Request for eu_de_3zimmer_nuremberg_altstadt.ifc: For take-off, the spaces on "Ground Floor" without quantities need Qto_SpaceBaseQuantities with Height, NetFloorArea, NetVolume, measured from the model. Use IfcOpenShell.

First a look at what the model holds.

```python
import ifcopenshell
import ifcopenshell.util.element
import ifcopenshell.util.unit

model = ifcopenshell.open("eu_de_3zimmer_nuremberg_altstadt.ifc")
print(model.schema)
for unit_type in ("LENGTHUNIT", "AREAUNIT", "VOLUMEUNIT"):
    print(unit_type, ifcopenshell.util.unit.calculate_unit_scale(model, unit_type))
storey = next(s for s in model.by_type("IfcBuildingStorey") if s.Name == "Ground Floor")
spaces = [e for e in ifcopenshell.util.element.get_decomposition(storey) if e.is_a("IfcSpace")]
for e in sorted(spaces, key=lambda e: e.id()):
    print(e.id(), e.is_a(), e.Name, list(ifcopenshell.util.element.get_psets(e, qtos_only=True)), sep=" | ")
```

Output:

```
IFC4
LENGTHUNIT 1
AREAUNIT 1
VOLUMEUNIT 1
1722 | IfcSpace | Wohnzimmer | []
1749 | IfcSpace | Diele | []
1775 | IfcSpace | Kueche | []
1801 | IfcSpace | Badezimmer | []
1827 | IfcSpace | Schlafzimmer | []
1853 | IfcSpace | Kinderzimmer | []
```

```python
import ifcopenshell
import ifcopenshell.api.pset
import ifcopenshell.geom
import ifcopenshell.util.element
import ifcopenshell.util.shape
import ifcopenshell.util.unit

model = ifcopenshell.open("eu_de_3zimmer_nuremberg_altstadt.ifc")
unit_scale = ifcopenshell.util.unit.calculate_unit_scale(model)
area_scale = ifcopenshell.util.unit.calculate_unit_scale(model, "AREAUNIT")
volume_scale = ifcopenshell.util.unit.calculate_unit_scale(model, "VOLUMEUNIT")
settings = ifcopenshell.geom.settings()

storey = next(s for s in model.by_type("IfcBuildingStorey") if s.Name == "Ground Floor")
spaces = [e for e in ifcopenshell.util.element.get_decomposition(storey) if e.is_a("IfcSpace")]

for e in sorted(spaces, key=lambda e: e.id()):
    if ifcopenshell.util.element.get_psets(e, qtos_only=True, should_inherit=False):
        continue
    # Geometry comes back in metres, in the element's own axes.
    shape = ifcopenshell.geom.create_shape(settings, e)
    values = {
        "Height": ifcopenshell.util.shape.get_z(shape.geometry) / unit_scale,
        "NetFloorArea": ifcopenshell.util.shape.get_footprint_area(shape.geometry) / area_scale,
        "NetVolume": ifcopenshell.util.shape.get_volume(shape.geometry) / volume_scale,
    }
    qto = ifcopenshell.api.pset.add_qto(model, product=e, name="Qto_SpaceBaseQuantities")
    ifcopenshell.api.pset.edit_qto(model, qto=qto, properties=values)
    print(e.id(), {k: round(v, 3) for k, v in values.items()})

model.write("eu_de_3zimmer_nuremberg_altstadt_rev.ifc")
```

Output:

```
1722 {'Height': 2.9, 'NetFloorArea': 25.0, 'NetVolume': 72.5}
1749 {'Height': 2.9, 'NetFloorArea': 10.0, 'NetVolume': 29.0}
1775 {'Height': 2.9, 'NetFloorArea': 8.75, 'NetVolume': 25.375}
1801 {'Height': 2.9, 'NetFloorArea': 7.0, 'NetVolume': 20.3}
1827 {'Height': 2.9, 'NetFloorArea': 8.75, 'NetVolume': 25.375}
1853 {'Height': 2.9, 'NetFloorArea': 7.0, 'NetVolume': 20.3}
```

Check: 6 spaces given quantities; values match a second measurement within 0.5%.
